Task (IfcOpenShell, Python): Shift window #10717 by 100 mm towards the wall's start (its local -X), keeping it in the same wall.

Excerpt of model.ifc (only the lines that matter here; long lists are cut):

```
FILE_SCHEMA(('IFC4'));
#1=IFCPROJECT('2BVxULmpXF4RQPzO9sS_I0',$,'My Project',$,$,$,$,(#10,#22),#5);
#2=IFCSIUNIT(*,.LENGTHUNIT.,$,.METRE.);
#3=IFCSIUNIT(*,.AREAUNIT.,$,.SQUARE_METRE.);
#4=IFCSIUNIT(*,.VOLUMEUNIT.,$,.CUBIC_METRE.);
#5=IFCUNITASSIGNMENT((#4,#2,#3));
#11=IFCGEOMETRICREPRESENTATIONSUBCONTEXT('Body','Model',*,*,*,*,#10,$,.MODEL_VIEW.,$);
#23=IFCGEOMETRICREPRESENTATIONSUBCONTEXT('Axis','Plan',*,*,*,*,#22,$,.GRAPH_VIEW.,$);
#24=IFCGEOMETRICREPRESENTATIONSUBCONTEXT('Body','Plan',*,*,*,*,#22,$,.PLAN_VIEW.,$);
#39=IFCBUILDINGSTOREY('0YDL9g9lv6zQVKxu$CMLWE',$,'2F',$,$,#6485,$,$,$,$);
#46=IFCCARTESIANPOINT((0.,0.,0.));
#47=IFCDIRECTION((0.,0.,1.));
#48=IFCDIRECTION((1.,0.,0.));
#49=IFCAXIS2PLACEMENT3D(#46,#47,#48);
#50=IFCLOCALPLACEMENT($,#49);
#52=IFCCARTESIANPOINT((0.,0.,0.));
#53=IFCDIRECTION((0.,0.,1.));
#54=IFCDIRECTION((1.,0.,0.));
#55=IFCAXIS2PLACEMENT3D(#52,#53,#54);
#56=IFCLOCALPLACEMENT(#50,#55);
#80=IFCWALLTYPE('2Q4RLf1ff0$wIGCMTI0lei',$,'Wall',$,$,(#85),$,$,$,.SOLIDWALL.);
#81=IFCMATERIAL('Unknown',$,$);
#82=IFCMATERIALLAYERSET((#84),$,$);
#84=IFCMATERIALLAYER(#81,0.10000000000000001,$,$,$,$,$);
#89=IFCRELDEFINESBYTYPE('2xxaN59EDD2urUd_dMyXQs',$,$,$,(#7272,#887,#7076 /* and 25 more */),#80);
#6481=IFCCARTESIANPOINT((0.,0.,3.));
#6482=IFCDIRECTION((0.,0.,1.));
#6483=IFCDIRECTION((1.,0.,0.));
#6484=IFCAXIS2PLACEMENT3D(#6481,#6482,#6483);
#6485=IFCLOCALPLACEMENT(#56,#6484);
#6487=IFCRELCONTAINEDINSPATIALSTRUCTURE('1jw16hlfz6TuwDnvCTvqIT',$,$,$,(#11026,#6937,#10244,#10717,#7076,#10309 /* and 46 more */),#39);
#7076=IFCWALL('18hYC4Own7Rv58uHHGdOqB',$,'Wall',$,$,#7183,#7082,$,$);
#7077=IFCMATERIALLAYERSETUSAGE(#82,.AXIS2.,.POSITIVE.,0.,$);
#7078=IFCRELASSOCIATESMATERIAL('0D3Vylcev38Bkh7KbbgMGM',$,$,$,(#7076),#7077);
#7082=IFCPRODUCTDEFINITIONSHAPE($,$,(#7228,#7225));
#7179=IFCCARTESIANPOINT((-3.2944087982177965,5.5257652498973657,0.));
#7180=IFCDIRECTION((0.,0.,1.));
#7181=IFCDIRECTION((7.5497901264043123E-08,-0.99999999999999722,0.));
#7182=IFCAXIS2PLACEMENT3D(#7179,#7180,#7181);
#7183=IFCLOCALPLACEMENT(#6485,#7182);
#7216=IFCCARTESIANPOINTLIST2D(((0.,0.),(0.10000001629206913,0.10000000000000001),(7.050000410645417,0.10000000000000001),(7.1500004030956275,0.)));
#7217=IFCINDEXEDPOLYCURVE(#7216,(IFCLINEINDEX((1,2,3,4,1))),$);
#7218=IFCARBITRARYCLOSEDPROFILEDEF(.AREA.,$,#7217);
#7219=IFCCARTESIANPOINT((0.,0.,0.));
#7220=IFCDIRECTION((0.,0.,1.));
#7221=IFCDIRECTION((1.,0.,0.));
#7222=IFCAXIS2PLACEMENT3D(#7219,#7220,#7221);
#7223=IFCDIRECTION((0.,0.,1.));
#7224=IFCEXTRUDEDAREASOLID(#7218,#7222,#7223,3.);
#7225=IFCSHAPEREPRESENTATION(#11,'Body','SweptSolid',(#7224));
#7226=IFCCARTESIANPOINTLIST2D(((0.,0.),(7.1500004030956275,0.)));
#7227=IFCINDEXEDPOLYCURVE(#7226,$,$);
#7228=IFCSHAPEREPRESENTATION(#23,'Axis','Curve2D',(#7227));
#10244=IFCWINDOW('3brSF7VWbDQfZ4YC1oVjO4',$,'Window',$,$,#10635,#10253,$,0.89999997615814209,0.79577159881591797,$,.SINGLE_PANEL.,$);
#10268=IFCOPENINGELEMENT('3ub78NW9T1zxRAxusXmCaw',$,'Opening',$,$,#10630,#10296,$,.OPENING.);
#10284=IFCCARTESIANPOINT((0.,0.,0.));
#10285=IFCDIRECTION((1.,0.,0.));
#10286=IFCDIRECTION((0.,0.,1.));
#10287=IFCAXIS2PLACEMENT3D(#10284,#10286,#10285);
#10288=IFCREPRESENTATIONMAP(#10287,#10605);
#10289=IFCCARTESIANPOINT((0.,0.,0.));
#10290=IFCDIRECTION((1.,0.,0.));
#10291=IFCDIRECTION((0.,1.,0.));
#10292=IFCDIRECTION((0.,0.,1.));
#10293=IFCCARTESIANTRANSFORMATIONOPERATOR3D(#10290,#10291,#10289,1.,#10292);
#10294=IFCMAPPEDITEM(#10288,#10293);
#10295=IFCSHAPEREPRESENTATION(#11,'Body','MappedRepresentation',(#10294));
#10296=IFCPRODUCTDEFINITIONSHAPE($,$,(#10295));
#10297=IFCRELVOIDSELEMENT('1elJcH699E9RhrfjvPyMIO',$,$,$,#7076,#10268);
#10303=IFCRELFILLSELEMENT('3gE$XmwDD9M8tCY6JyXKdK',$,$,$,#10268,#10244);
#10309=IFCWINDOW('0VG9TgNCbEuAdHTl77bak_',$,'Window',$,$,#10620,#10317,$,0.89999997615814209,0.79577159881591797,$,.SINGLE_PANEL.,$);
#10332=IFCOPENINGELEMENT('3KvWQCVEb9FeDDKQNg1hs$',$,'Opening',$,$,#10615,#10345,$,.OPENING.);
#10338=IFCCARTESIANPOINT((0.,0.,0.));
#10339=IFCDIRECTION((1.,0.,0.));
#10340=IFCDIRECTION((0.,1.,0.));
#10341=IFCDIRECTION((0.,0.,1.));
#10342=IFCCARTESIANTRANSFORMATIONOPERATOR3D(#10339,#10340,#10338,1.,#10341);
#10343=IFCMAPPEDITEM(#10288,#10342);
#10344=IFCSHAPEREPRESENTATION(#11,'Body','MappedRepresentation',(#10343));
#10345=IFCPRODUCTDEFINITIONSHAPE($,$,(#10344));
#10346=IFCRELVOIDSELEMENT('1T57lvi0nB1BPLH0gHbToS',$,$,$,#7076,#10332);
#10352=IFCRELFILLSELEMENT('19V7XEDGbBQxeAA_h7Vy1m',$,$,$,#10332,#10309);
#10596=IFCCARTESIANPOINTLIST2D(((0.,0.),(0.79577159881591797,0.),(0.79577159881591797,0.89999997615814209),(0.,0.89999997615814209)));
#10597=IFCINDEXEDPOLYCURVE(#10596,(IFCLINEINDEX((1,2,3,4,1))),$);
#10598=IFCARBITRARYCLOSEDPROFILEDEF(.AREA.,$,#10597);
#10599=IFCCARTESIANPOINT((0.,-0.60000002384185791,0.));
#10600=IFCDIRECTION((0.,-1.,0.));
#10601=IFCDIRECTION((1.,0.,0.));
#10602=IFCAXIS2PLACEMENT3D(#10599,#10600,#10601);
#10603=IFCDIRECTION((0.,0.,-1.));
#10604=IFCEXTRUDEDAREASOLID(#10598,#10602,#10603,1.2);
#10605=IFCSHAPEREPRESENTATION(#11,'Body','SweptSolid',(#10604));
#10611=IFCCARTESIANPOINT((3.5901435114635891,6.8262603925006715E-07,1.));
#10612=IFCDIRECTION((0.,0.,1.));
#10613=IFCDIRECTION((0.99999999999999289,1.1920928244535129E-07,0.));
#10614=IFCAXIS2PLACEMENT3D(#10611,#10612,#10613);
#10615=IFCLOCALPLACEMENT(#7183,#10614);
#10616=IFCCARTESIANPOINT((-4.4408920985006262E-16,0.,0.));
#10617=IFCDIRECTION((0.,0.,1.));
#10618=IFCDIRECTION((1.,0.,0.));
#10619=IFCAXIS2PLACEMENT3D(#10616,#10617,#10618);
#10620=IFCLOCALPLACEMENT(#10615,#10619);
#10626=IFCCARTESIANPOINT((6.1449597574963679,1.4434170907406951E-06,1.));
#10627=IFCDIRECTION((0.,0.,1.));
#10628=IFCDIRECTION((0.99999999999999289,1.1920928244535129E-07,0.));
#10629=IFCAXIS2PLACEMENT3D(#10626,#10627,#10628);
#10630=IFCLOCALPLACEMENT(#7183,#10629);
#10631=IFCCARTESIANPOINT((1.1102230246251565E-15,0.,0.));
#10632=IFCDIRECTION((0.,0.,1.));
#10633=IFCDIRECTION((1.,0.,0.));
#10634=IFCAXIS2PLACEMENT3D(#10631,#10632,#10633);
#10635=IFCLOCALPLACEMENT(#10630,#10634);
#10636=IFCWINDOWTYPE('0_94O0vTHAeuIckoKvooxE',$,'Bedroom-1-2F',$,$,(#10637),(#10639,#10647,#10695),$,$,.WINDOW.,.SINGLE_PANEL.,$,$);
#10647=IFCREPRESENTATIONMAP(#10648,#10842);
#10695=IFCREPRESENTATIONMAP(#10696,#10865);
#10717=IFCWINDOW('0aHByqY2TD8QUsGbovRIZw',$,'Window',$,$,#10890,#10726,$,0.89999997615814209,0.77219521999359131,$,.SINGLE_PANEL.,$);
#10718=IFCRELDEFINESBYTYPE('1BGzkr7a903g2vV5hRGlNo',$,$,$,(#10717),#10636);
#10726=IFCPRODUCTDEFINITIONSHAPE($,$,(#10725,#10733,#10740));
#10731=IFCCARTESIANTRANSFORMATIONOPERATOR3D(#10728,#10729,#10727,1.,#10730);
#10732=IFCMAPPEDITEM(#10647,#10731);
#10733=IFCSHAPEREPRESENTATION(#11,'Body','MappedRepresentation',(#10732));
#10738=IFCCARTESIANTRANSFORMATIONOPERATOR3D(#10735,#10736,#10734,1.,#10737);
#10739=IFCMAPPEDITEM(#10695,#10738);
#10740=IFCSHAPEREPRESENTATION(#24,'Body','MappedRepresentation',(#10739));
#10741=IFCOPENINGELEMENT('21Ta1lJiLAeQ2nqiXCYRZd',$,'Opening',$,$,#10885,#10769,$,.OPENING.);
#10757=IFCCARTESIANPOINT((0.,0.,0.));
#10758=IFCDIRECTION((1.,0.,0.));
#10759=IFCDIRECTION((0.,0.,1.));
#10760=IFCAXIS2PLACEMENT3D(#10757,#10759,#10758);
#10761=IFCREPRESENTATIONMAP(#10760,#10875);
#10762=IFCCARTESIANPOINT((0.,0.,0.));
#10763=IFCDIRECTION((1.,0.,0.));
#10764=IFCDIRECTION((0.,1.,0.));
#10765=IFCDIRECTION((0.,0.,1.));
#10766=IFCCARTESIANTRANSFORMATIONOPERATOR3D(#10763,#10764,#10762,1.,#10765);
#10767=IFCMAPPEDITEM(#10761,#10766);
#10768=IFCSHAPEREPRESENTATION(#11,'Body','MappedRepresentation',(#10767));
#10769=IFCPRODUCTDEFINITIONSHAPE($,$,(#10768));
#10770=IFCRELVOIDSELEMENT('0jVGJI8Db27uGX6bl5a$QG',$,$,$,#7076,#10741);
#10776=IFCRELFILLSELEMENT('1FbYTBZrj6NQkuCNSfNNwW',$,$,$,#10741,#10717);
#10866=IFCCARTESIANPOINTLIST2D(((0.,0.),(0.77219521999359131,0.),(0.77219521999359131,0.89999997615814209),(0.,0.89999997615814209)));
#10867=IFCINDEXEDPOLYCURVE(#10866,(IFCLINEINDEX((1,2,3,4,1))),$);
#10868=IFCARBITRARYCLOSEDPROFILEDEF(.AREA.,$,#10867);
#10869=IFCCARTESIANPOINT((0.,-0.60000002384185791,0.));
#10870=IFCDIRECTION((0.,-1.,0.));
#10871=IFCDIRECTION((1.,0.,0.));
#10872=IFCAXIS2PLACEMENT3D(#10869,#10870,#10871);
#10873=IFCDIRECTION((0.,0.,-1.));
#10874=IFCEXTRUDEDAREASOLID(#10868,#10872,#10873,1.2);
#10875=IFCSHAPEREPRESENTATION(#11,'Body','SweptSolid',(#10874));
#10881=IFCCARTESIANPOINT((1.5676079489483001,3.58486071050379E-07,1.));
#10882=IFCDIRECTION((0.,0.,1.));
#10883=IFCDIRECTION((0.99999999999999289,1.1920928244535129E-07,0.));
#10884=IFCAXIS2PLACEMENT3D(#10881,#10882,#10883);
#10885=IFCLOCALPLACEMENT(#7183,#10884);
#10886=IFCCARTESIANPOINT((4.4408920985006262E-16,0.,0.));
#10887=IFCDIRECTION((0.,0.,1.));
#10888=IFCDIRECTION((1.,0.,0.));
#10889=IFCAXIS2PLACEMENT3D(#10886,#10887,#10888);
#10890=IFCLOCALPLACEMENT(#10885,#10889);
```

```python
import ifcopenshell
import ifcopenshell.api.geometry
import ifcopenshell.util.placement
import ifcopenshell.util.unit

model = ifcopenshell.open("model.ifc")
unit_scale = ifcopenshell.util.unit.calculate_unit_scale(model)

window = model.by_guid("0aHByqY2TD8QUsGbovRIZw")
opening = window.FillsVoids[0].RelatingOpeningElement
wall = opening.VoidsElements[0].RelatingBuildingElement

wall_matrix = ifcopenshell.util.placement.get_local_placement(wall.ObjectPlacement)
shift = wall_matrix[:3, 0] * -0.1 / unit_scale
before = ifcopenshell.util.placement.get_local_placement(window.ObjectPlacement)[:3, 3].copy()

# The window is placed relative to its opening, so it follows when the opening moves.
matrix = ifcopenshell.util.placement.get_local_placement(opening.ObjectPlacement)
matrix[:3, 3] += shift
ifcopenshell.api.geometry.edit_object_placement(
    model, product=opening, matrix=matrix, is_si=False, should_transform_children=True
)

after = ifcopenshell.util.placement.get_local_placement(window.ObjectPlacement)[:3, 3]
print("window moved by", (after - before).round(3) + 0.0)

model.write("model_rev.ifc")
```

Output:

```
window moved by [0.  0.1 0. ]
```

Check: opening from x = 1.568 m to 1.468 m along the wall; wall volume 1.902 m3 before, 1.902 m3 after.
